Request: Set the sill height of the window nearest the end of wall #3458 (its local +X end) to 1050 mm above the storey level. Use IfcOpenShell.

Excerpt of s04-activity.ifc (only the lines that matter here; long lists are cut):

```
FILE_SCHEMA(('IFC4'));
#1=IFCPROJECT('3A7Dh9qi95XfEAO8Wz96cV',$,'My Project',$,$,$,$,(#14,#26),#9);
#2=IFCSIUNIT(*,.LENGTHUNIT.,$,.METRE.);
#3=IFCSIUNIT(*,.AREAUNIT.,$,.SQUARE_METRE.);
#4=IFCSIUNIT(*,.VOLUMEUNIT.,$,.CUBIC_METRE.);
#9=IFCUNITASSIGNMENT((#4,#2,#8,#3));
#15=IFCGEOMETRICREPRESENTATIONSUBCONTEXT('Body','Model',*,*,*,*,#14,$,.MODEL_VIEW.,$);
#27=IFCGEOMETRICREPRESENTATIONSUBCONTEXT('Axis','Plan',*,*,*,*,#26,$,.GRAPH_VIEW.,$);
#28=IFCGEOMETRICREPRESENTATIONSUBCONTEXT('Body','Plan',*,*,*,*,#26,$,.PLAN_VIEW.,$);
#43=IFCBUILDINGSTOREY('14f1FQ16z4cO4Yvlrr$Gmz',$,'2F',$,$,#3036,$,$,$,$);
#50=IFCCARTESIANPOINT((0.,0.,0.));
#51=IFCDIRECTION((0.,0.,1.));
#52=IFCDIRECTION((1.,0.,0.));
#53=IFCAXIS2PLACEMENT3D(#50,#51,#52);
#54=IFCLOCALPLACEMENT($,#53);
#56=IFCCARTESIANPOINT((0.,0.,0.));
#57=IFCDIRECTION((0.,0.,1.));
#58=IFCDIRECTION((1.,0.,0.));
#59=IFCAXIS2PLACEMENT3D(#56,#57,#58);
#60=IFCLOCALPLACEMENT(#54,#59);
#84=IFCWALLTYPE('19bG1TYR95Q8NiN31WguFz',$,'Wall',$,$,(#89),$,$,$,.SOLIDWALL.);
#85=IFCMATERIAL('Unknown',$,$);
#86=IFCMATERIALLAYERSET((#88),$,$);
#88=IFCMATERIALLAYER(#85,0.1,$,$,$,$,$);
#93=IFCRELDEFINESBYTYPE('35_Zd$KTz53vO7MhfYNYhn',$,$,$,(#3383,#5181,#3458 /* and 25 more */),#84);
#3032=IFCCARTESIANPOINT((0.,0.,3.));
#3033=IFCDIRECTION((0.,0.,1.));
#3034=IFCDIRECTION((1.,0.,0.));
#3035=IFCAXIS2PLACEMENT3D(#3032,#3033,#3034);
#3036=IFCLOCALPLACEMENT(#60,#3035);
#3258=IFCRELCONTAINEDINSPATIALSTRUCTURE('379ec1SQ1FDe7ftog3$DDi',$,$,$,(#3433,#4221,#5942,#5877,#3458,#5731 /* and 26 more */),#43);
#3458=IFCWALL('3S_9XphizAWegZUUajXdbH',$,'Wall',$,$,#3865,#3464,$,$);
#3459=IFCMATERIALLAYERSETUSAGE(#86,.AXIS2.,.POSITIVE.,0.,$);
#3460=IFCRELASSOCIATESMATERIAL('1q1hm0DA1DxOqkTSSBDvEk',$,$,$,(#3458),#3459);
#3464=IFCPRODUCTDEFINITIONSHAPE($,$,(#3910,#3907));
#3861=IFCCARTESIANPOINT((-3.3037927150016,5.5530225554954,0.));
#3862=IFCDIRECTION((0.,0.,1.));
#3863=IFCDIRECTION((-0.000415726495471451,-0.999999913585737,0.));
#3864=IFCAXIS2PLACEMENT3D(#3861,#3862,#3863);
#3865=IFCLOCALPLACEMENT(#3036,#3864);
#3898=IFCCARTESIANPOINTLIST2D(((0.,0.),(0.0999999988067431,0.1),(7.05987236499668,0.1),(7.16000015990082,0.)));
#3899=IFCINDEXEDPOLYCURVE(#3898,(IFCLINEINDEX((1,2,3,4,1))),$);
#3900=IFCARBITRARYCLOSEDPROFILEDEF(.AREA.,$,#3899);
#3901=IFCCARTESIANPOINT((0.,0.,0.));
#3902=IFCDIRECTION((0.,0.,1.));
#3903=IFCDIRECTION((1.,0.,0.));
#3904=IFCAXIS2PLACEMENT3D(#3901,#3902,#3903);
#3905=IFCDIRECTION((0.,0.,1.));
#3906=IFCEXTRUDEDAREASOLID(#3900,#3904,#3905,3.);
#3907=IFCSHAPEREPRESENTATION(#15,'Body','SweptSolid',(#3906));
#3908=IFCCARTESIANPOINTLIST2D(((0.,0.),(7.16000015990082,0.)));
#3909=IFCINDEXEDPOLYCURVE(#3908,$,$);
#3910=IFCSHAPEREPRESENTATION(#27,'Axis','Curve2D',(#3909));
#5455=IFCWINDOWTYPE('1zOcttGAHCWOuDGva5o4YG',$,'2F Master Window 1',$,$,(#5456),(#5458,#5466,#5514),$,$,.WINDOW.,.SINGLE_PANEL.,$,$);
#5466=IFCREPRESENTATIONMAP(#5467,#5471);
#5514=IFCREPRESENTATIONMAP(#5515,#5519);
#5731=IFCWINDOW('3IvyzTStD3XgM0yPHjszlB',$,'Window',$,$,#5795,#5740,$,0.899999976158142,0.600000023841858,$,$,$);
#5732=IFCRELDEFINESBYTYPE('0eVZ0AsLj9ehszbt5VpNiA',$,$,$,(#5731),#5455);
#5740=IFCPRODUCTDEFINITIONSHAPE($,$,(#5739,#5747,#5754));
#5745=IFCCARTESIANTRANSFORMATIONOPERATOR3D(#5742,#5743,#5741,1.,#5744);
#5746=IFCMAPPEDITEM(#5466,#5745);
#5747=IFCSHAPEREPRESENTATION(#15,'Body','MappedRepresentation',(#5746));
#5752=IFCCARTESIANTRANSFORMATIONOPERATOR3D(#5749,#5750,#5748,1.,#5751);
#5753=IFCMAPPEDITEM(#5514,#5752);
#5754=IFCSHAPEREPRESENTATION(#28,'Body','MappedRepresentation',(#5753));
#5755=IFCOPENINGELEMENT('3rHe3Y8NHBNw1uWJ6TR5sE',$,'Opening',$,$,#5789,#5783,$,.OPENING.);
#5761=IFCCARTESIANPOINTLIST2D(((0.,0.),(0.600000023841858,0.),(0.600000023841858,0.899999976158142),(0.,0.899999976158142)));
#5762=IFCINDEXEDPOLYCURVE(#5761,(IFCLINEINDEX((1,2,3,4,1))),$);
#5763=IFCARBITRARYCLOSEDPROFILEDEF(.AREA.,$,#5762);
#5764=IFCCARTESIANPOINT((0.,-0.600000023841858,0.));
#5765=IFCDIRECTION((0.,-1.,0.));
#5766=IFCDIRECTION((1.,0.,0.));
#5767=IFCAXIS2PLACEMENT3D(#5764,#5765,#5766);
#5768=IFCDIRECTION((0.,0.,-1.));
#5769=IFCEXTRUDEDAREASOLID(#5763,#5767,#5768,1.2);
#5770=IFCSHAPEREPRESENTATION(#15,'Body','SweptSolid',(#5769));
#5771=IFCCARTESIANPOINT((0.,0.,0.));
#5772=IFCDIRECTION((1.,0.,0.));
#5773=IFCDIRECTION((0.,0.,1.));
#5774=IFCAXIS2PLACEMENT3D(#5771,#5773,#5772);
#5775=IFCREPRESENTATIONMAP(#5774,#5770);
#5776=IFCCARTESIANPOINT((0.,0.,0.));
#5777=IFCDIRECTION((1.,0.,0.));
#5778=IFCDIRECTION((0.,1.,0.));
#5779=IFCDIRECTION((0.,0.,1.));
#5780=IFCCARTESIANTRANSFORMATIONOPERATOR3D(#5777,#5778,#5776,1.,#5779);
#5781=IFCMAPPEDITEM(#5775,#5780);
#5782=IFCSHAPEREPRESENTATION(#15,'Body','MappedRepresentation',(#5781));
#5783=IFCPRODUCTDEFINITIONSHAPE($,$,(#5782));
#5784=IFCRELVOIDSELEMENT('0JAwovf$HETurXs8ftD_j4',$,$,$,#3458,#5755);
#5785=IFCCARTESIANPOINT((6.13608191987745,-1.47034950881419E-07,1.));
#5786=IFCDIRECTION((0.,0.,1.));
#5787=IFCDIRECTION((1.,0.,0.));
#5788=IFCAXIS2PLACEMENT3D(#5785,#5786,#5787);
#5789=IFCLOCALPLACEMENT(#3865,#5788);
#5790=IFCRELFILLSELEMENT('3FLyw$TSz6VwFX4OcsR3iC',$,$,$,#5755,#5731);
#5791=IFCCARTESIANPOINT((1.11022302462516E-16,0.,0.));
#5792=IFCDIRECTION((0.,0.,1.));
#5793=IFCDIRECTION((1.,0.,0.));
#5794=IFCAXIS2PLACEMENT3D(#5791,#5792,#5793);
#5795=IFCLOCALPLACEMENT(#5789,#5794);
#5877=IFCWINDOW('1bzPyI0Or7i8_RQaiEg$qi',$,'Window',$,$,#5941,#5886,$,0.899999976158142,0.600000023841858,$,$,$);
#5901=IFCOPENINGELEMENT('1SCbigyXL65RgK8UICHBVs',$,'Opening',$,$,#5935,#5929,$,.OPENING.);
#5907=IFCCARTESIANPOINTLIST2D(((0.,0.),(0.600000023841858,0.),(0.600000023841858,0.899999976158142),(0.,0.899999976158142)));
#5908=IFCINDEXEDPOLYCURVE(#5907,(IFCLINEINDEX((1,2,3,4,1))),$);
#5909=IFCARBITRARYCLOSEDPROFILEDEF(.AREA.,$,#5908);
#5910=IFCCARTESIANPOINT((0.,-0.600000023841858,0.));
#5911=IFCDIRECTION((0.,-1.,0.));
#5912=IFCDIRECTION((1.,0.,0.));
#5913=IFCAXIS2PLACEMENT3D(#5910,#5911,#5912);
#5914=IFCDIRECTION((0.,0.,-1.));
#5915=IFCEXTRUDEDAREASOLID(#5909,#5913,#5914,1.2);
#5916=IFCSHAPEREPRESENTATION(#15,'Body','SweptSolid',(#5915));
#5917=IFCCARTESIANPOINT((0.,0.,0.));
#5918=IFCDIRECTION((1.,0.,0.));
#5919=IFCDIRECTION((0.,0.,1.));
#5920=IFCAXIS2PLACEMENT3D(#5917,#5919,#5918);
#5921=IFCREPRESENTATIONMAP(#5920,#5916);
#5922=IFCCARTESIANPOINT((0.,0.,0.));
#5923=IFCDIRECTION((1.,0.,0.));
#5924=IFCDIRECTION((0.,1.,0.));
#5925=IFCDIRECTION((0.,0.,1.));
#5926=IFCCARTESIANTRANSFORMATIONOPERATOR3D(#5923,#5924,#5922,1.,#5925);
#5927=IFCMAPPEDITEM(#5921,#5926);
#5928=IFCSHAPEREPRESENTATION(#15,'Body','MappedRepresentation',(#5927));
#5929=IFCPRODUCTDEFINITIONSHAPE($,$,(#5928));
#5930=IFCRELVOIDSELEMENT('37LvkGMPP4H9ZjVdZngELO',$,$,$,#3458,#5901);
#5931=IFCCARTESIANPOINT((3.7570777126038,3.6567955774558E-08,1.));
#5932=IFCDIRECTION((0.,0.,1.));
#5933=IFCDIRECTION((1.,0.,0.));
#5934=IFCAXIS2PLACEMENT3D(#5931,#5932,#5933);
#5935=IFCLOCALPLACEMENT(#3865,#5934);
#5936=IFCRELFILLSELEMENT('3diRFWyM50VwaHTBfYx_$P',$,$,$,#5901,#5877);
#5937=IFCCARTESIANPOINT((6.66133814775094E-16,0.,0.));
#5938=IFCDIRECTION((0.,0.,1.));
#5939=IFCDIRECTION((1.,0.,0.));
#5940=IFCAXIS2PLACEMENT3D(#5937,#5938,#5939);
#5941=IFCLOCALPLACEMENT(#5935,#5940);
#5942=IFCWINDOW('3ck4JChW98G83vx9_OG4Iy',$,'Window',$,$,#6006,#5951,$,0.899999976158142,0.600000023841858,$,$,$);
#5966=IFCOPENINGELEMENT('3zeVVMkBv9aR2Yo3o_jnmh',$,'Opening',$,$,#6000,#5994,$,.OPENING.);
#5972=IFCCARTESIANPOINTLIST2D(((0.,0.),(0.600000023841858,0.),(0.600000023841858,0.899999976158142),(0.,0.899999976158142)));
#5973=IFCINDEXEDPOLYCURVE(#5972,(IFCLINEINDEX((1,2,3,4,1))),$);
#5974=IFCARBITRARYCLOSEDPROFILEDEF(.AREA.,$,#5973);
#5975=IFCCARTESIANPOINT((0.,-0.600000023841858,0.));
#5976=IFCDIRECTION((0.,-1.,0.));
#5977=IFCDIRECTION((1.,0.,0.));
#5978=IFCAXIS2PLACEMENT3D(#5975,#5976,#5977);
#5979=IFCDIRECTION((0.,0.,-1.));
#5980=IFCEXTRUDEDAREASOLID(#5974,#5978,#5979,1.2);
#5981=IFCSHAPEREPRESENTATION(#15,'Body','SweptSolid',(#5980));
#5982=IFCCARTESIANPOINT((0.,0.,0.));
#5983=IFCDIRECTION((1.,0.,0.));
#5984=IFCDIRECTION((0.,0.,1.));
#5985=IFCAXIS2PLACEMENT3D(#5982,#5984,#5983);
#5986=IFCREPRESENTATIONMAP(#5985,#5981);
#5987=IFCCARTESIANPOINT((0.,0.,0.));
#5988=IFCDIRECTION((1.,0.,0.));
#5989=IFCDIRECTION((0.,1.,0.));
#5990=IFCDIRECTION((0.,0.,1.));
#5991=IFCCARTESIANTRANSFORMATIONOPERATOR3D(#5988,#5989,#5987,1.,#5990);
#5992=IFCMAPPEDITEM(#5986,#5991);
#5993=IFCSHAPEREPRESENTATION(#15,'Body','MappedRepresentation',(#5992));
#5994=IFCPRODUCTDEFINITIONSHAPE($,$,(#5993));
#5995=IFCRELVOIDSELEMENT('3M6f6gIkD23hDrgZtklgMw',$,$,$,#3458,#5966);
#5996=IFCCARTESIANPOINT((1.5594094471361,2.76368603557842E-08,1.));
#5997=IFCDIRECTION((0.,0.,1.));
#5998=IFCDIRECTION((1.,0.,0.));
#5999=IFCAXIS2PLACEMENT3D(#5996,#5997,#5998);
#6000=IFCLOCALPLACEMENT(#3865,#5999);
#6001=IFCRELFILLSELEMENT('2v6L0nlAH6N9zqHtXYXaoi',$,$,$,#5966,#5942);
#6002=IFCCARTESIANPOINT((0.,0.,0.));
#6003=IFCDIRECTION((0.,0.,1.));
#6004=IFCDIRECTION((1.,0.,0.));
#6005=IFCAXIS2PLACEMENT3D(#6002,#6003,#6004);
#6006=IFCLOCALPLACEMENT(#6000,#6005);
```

```python
import numpy as np
import ifcopenshell
import ifcopenshell.api.geometry
import ifcopenshell.geom
import ifcopenshell.util.element
import ifcopenshell.util.placement
import ifcopenshell.util.shape
import ifcopenshell.util.unit

model = ifcopenshell.open("s04-activity.ifc")
unit_scale = ifcopenshell.util.unit.calculate_unit_scale(model)

window = model.by_id(5731)
opening = window.FillsVoids[0].RelatingOpeningElement
storey = ifcopenshell.util.element.get_container(window, ifc_class="IfcBuildingStorey")
level = ifcopenshell.util.placement.get_local_placement(storey.ObjectPlacement)[2, 3]

# The opening's origin need not be at the sill, so measure its lowest point.
shape = ifcopenshell.geom.create_shape(ifcopenshell.geom.settings(), opening)
bottom = ifcopenshell.util.shape.get_shape_bottom_elevation(shape, shape.geometry) / unit_scale
dz = level + 1.05 / unit_scale - bottom

shift = np.array([0.0, 0.0, dz])
# The window is placed relative to its opening, so it follows when the opening moves.
matrix = ifcopenshell.util.placement.get_local_placement(opening.ObjectPlacement)
matrix[:3, 3] += shift
ifcopenshell.api.geometry.edit_object_placement(
    model, product=opening, matrix=matrix, is_si=False, should_transform_children=True
)

print(f"moved by {dz * unit_scale:+.3f} m")

model.write("s04-activity-out.ifc")
```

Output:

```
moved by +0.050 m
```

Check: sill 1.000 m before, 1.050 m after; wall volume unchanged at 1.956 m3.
